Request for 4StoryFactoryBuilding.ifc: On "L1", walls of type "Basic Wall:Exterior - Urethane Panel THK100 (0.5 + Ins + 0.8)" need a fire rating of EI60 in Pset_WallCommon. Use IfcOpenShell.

First a look at what the model holds.

```python
import ifcopenshell
import ifcopenshell.util.element

model = ifcopenshell.open("4StoryFactoryBuilding.ifc")
print(model.schema)
storey = next(s for s in model.by_type("IfcBuildingStorey") if s.Name == "L1")
walls = [e for e in ifcopenshell.util.element.get_decomposition(storey) if e.is_a("IfcWall")]
seen = {}
for e in walls:
    element_type = ifcopenshell.util.element.get_type(e)
    key = (element_type.Name if element_type != e and element_type else None, ifcopenshell.util.element.get_pset(e, "Pset_WallCommon", "FireRating"))
    seen[key] = seen.get(key, 0) + 1
for (name, value), count in sorted(seen.items(), key=str):
    print(count, "x", name, "|", value)
```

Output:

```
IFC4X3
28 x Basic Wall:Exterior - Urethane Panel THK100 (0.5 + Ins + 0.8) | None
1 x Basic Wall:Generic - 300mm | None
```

```python
import ifcopenshell
import ifcopenshell.api.pset
import ifcopenshell.util.element

model = ifcopenshell.open("4StoryFactoryBuilding.ifc")

storey = next(s for s in model.by_type("IfcBuildingStorey") if s.Name == "L1")
walls = [e for e in ifcopenshell.util.element.get_decomposition(storey) if e.is_a("IfcWall")]

count = 0
for e in walls:
    element_type = ifcopenshell.util.element.get_type(e)
    if element_type in (None, e) or element_type.Name != "Basic Wall:Exterior - Urethane Panel THK100 (0.5 + Ins + 0.8)":
        continue
    # add_pset returns the element's existing set when there is one.
    pset = ifcopenshell.api.pset.add_pset(model, product=e, name="Pset_WallCommon")
    ifcopenshell.api.pset.edit_pset(model, pset=pset, properties={"FireRating": "EI60"})
    count += 1

print(count, "walls updated")

model.write("4StoryFactoryBuilding-out.ifc")
```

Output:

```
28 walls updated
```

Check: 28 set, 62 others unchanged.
